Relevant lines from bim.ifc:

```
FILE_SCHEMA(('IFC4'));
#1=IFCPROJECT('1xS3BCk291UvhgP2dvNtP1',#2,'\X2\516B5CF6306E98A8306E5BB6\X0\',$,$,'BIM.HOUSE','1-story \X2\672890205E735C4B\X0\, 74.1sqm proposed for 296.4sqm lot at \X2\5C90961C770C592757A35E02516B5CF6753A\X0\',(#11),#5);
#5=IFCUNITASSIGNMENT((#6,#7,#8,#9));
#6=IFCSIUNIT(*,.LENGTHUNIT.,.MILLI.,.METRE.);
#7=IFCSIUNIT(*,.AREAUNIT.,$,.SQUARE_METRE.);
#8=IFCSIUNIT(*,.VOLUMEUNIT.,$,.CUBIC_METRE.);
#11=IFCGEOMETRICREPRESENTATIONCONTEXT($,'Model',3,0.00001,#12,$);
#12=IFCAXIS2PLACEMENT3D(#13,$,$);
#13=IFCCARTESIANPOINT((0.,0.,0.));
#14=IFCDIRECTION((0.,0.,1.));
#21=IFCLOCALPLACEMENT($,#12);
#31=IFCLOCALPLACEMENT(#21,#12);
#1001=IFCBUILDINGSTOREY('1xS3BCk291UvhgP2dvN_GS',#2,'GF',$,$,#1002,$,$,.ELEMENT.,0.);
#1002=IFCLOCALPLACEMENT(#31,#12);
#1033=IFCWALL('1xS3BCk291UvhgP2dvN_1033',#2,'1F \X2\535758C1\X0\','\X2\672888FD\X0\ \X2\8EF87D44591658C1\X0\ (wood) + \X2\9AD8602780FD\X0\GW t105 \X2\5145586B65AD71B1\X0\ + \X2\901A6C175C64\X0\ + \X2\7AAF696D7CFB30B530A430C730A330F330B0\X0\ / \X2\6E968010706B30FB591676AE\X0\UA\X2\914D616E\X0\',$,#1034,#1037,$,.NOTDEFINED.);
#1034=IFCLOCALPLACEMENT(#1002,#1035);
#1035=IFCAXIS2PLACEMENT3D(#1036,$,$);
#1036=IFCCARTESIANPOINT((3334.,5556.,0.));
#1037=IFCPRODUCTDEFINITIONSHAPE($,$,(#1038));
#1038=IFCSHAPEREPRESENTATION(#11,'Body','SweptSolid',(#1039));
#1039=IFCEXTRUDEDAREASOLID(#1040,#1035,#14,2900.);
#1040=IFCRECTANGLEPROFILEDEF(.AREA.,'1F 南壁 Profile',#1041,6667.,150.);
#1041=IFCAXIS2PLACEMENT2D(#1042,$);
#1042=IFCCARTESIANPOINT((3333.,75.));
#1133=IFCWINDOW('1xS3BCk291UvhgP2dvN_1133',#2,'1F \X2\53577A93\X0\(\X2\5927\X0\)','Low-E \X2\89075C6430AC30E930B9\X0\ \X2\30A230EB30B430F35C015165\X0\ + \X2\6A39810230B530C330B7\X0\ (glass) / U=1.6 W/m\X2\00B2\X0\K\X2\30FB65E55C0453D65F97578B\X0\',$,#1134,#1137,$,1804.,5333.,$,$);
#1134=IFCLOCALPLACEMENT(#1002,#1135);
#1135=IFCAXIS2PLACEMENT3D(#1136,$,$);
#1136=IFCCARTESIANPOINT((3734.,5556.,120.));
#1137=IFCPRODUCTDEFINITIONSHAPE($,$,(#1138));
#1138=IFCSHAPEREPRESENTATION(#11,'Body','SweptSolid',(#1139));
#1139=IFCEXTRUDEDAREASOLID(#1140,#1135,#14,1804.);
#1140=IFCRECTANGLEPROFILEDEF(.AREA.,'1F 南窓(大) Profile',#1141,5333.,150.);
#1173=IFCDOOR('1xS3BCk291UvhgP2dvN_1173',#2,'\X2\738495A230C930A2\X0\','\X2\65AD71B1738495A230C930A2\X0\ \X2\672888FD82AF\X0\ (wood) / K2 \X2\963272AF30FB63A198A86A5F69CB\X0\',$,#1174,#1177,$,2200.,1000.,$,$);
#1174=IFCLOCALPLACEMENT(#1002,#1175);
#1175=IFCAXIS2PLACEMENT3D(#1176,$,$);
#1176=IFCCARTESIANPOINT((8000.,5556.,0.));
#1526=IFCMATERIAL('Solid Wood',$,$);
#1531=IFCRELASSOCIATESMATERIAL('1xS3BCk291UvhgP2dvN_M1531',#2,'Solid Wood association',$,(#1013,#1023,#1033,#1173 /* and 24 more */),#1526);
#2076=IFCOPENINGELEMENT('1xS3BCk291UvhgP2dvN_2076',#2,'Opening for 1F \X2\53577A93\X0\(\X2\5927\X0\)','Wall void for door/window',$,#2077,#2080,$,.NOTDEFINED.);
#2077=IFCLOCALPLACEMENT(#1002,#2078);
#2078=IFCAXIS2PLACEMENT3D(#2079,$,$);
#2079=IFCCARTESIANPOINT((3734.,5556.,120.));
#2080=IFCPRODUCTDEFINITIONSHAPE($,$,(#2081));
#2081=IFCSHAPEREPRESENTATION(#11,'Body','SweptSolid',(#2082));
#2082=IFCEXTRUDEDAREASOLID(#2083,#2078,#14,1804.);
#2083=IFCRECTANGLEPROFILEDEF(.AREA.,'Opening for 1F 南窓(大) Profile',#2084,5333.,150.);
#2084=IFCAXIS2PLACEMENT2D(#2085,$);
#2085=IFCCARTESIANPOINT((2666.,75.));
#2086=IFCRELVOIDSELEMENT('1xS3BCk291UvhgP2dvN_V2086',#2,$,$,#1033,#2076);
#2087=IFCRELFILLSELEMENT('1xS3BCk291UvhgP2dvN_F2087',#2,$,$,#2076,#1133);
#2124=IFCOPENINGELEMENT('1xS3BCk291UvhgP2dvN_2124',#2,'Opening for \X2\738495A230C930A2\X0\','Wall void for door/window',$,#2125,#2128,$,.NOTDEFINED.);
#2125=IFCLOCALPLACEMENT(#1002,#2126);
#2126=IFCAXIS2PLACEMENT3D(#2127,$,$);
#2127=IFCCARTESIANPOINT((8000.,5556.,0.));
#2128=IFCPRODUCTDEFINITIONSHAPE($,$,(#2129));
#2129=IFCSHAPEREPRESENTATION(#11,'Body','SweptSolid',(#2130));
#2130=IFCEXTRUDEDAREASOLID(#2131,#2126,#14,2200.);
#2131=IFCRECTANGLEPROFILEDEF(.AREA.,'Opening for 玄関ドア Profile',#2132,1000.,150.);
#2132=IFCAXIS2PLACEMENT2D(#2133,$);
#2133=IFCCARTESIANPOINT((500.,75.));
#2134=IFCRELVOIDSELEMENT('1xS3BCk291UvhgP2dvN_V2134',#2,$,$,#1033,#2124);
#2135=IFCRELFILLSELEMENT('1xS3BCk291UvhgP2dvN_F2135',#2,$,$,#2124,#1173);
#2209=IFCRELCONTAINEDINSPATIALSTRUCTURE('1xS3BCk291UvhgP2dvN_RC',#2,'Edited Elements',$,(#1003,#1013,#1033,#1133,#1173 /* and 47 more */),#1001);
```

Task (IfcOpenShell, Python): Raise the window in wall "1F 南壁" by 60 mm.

```python
import numpy as np
import ifcopenshell
import ifcopenshell.api.geometry
import ifcopenshell.util.placement
import ifcopenshell.util.unit

model = ifcopenshell.open("bim.ifc")
unit_scale = ifcopenshell.util.unit.calculate_unit_scale(model)

window = model.by_guid("1xS3BCk291UvhgP2dvN_1133")
opening = window.FillsVoids[0].RelatingOpeningElement
dz = 0.06 / unit_scale

shift = np.array([0.0, 0.0, dz])
# The window is not placed relative to its opening, so move both.
for product in (opening, window):
    matrix = ifcopenshell.util.placement.get_local_placement(product.ObjectPlacement)
    matrix[:3, 3] += shift
    ifcopenshell.api.geometry.edit_object_placement(model, product=product, matrix=matrix, is_si=False)

print(f"moved by {dz * unit_scale:+.3f} m")

model.write("bim_updated.ifc")
```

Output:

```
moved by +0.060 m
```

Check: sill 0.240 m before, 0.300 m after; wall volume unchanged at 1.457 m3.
